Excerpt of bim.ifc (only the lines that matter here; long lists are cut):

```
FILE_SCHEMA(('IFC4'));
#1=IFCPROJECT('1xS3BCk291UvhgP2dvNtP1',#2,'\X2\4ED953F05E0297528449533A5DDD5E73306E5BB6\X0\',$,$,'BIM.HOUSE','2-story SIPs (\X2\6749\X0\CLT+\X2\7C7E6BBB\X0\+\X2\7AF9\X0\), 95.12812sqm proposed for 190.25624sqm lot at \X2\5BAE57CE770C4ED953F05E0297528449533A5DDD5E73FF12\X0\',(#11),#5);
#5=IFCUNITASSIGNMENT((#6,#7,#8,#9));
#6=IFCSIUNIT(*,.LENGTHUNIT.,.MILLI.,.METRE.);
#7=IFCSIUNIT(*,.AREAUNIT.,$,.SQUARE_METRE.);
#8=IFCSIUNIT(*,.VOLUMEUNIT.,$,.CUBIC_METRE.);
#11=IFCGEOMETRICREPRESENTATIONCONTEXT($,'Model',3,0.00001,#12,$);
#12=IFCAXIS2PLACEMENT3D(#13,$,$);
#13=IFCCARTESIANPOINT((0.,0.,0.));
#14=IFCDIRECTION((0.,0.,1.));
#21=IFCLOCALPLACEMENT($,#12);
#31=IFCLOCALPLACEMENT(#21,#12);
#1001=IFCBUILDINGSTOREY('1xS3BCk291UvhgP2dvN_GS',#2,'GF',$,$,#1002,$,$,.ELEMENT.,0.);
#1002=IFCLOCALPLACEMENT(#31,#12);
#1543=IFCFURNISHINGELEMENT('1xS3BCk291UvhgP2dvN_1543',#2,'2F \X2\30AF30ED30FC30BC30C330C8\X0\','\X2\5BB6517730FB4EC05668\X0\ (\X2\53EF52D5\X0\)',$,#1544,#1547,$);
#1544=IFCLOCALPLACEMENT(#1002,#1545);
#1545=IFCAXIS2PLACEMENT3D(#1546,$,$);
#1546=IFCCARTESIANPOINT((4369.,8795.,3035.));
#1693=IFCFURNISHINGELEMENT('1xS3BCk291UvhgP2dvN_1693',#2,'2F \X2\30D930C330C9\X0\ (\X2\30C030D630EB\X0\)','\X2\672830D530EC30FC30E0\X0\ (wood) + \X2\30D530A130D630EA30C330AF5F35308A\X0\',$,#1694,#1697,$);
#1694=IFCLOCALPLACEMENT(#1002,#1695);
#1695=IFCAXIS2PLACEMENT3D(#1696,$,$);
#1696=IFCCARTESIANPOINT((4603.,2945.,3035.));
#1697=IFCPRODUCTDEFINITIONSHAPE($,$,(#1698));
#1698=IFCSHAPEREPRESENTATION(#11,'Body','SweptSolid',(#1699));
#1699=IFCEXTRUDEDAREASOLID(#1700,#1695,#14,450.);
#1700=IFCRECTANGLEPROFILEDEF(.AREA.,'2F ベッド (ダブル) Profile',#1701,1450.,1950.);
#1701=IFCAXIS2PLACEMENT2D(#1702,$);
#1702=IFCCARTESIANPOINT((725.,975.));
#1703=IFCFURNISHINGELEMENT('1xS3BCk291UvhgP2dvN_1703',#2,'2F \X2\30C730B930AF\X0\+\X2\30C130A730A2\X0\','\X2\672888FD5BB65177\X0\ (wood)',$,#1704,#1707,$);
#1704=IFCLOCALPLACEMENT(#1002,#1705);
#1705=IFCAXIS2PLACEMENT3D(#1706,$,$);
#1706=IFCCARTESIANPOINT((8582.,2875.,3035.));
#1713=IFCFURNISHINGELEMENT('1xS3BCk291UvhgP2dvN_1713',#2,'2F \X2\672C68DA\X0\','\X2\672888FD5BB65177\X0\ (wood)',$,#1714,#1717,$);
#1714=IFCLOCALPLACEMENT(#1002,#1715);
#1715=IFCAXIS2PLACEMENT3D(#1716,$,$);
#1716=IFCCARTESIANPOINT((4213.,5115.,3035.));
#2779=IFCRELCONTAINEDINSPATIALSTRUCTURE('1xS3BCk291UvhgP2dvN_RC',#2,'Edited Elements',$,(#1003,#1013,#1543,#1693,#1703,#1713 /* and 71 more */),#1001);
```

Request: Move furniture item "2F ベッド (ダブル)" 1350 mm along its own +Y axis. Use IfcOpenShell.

```python
import ifcopenshell
import ifcopenshell.api.geometry
import ifcopenshell.util.placement

model = ifcopenshell.open("bim.ifc")

item = model.by_guid("1xS3BCk291UvhgP2dvN_1693")
matrix = ifcopenshell.util.placement.get_local_placement(item.ObjectPlacement)
matrix[:3, 3] += matrix[:3, 1] * 1350.0
ifcopenshell.api.geometry.edit_object_placement(model, product=item, matrix=matrix, is_si=False)

print(ifcopenshell.util.placement.get_local_placement(item.ObjectPlacement).round(3) + 0.0)

model.write("bim-out.ifc")
```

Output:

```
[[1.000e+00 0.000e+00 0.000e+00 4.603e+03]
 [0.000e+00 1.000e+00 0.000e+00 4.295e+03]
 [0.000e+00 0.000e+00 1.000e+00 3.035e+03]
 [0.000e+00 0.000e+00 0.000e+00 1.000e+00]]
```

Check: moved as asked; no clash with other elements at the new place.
